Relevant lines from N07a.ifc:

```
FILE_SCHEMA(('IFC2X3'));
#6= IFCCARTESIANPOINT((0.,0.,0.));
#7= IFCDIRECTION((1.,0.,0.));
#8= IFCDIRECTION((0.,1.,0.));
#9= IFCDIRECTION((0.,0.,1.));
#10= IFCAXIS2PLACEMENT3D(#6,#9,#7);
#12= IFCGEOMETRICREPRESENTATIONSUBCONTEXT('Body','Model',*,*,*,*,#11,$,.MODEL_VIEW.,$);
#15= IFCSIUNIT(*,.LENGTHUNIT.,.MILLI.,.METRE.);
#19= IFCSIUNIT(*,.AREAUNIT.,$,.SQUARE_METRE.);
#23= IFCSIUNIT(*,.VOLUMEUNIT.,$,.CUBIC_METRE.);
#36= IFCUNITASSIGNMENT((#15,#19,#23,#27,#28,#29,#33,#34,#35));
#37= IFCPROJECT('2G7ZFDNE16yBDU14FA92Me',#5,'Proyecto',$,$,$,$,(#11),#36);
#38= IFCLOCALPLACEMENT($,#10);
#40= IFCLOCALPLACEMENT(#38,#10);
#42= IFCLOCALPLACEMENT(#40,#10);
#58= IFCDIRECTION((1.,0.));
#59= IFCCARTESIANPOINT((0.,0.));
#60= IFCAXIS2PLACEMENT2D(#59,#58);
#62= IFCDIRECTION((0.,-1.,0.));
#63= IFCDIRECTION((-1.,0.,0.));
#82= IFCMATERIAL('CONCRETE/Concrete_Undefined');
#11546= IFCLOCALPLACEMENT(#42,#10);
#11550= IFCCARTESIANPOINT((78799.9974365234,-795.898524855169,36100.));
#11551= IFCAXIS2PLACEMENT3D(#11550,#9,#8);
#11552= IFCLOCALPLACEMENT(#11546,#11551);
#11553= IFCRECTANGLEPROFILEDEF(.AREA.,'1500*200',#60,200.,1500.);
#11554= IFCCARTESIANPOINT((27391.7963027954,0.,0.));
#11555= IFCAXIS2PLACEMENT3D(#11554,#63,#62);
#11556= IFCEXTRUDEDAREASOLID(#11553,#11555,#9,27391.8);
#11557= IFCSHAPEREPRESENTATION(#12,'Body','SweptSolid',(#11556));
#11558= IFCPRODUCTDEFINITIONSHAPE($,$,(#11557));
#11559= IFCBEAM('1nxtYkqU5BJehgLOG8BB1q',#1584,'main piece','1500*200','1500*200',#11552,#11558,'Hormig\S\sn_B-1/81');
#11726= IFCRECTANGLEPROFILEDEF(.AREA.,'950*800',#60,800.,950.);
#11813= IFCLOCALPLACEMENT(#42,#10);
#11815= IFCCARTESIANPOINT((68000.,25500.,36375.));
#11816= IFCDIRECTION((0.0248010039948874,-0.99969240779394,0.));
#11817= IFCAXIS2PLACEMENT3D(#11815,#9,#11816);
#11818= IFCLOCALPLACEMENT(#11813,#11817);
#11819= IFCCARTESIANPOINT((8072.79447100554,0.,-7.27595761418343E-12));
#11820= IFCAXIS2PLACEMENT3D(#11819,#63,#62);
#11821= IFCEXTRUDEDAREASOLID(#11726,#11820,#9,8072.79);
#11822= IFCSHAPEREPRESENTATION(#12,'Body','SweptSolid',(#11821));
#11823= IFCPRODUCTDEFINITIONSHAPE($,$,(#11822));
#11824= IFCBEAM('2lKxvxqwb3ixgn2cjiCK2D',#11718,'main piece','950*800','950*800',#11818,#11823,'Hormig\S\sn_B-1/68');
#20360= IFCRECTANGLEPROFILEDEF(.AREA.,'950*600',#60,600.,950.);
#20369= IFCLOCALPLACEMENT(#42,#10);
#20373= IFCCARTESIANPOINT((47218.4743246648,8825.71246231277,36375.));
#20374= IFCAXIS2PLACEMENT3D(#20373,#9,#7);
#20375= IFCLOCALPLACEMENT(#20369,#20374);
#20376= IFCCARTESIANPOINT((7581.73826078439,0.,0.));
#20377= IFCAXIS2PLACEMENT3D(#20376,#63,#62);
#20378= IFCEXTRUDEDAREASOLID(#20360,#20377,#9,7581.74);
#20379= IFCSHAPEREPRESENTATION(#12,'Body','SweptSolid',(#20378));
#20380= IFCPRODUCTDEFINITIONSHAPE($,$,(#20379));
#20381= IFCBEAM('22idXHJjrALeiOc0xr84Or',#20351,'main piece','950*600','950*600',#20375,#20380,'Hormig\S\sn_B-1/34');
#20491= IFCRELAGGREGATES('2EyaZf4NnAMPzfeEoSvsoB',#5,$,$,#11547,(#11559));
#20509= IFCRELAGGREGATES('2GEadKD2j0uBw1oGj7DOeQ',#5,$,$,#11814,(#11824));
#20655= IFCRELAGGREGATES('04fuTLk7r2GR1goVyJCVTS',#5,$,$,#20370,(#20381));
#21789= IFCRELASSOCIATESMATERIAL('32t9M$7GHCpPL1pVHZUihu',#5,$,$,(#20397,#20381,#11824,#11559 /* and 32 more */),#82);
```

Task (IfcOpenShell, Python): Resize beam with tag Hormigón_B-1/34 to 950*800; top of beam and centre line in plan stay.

```python
import ifcopenshell
import ifcopenshell.util.element
import ifcopenshell.util.representation

model = ifcopenshell.open("N07a.ifc")

member = model.by_guid("22idXHJjrALeiOc0xr84Or")
source = next(p for p in model.by_type("IfcRectangleProfileDef") if p.ProfileName == "950*800")

body = ifcopenshell.util.representation.get_representation(member, "Model", "Body")
solid = body.Items[0]
old_profile = solid.SweptArea

# Copy the section's sizes but keep this member's own profile position.
profile = ifcopenshell.util.element.copy(model, source)
# Profiles are centred, so shift by half the change in depth to hold the top.
shift = (old_profile.YDim - profile.YDim) / 2
x, y = old_profile.Position.Location.Coordinates
up = (0.0, 1.0)  # upwards, in the solid's own plane
location = model.createIfcCartesianPoint((x + up[0] * shift, y + up[1] * shift))
profile.Position = model.createIfcAxis2Placement2D(location, old_profile.Position.RefDirection)
solid.SweptArea = profile
if not model.get_total_inverses(old_profile):
    ifcopenshell.util.element.remove_deep2(model, old_profile)
member.Description = member.Description.replace("950*600", "950*800")
member.ObjectType = member.ObjectType.replace("950*600", "950*800")

print(solid.SweptArea)

model.write("N07a_v2.ifc")
```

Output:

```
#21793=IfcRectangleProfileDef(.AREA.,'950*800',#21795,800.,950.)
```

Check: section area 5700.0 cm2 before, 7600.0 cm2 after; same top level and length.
